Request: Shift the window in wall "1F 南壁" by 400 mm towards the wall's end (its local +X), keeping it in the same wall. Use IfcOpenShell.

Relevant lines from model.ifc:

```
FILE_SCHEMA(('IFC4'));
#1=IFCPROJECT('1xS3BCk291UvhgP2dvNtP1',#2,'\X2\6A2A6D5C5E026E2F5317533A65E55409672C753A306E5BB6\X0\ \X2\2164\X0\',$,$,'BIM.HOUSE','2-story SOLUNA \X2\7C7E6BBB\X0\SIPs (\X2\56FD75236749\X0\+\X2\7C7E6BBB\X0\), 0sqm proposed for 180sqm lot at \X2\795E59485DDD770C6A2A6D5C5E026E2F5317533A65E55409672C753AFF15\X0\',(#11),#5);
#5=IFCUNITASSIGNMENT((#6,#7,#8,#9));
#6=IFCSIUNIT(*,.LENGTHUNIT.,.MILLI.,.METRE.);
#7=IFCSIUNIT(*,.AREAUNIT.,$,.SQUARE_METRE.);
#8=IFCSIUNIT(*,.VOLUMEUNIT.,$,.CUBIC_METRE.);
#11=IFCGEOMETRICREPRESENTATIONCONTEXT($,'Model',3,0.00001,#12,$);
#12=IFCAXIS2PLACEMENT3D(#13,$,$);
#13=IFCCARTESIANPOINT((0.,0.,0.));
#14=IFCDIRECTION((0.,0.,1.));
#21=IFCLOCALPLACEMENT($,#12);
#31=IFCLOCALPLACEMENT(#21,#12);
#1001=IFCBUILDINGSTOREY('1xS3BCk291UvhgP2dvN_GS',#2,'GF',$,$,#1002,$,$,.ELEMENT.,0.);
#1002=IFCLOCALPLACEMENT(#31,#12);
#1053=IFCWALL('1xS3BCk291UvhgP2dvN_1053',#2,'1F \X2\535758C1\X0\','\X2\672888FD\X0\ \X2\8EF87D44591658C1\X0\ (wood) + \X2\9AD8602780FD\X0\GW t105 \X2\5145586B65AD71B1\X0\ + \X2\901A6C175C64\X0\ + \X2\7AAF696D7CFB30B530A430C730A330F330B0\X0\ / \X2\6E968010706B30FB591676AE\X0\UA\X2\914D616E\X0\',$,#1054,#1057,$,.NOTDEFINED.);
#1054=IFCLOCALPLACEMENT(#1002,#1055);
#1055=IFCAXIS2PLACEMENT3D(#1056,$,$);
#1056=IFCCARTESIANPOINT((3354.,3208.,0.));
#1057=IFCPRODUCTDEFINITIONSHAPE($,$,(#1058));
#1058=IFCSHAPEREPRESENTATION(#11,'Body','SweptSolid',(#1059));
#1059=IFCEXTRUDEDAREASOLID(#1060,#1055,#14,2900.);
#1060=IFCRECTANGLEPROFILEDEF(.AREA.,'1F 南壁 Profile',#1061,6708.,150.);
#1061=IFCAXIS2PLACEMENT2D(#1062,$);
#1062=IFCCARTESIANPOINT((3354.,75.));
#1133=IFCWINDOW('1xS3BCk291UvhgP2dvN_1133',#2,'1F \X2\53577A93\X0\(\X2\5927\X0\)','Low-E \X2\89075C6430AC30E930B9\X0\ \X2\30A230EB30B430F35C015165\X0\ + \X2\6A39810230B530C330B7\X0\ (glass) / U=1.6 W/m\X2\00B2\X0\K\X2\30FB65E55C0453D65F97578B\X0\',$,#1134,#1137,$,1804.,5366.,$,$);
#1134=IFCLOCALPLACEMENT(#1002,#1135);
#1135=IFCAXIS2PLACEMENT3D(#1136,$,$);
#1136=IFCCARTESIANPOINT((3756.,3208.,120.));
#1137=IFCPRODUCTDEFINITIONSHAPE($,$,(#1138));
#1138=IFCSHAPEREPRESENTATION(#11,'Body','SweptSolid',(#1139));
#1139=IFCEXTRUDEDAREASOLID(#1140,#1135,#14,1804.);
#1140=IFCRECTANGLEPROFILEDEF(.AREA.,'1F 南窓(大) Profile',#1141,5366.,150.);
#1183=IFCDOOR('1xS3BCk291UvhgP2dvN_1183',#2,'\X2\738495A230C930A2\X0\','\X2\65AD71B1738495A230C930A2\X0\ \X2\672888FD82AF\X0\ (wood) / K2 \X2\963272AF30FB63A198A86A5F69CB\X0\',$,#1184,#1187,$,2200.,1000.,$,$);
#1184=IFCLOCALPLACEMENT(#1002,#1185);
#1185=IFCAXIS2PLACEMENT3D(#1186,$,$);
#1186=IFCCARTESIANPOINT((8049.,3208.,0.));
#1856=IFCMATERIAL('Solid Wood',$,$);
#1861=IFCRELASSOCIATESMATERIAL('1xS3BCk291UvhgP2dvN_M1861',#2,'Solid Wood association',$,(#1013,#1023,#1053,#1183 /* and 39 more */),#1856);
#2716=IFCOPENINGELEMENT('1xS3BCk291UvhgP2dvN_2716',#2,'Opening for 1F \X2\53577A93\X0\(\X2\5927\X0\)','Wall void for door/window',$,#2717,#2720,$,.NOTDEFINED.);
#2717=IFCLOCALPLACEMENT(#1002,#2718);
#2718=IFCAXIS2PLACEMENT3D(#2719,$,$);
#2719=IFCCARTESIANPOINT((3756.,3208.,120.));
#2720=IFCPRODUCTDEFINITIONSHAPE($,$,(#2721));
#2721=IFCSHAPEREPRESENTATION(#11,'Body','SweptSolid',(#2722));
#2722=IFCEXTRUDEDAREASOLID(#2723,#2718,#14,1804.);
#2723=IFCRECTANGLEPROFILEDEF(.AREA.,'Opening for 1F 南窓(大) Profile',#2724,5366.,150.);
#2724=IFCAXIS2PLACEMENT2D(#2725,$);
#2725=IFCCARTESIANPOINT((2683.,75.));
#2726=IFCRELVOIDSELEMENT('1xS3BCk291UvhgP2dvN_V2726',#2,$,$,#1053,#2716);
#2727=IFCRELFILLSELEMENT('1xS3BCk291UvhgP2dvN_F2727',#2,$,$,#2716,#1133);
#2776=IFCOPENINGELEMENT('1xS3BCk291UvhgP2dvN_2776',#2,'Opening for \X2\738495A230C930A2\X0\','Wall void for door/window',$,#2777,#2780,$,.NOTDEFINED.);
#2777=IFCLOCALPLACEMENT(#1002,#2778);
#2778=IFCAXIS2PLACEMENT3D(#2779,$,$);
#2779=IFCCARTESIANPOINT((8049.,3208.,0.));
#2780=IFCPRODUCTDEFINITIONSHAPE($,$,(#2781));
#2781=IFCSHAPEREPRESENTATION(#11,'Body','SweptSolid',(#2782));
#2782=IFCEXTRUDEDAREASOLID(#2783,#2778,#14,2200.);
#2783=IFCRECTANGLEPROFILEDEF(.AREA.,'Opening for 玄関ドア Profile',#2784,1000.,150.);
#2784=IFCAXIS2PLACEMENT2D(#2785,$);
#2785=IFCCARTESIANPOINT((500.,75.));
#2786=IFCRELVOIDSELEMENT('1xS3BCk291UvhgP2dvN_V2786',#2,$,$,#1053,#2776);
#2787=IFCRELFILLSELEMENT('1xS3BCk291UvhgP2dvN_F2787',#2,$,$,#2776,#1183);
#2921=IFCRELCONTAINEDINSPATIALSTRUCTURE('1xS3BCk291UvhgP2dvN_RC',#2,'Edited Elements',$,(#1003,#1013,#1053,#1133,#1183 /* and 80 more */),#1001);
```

```python
import ifcopenshell
import ifcopenshell.api.geometry
import ifcopenshell.util.placement
import ifcopenshell.util.unit

model = ifcopenshell.open("model.ifc")
unit_scale = ifcopenshell.util.unit.calculate_unit_scale(model)

window = model.by_id(1133)
opening = window.FillsVoids[0].RelatingOpeningElement
wall = opening.VoidsElements[0].RelatingBuildingElement

wall_matrix = ifcopenshell.util.placement.get_local_placement(wall.ObjectPlacement)
shift = wall_matrix[:3, 0] * 0.4 / unit_scale
before = ifcopenshell.util.placement.get_local_placement(window.ObjectPlacement)[:3, 3].copy()

# The window is not placed relative to its opening, so move both.
for product in (opening, window):
    matrix = ifcopenshell.util.placement.get_local_placement(product.ObjectPlacement)
    matrix[:3, 3] += shift
    ifcopenshell.api.geometry.edit_object_placement(model, product=product, matrix=matrix, is_si=False)

after = ifcopenshell.util.placement.get_local_placement(window.ObjectPlacement)[:3, 3]
print("window moved by", (after - before).round(3) + 0.0)

model.write("model_updated.ifc")
```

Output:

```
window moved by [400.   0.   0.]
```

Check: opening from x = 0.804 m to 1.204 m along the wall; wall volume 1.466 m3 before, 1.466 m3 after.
